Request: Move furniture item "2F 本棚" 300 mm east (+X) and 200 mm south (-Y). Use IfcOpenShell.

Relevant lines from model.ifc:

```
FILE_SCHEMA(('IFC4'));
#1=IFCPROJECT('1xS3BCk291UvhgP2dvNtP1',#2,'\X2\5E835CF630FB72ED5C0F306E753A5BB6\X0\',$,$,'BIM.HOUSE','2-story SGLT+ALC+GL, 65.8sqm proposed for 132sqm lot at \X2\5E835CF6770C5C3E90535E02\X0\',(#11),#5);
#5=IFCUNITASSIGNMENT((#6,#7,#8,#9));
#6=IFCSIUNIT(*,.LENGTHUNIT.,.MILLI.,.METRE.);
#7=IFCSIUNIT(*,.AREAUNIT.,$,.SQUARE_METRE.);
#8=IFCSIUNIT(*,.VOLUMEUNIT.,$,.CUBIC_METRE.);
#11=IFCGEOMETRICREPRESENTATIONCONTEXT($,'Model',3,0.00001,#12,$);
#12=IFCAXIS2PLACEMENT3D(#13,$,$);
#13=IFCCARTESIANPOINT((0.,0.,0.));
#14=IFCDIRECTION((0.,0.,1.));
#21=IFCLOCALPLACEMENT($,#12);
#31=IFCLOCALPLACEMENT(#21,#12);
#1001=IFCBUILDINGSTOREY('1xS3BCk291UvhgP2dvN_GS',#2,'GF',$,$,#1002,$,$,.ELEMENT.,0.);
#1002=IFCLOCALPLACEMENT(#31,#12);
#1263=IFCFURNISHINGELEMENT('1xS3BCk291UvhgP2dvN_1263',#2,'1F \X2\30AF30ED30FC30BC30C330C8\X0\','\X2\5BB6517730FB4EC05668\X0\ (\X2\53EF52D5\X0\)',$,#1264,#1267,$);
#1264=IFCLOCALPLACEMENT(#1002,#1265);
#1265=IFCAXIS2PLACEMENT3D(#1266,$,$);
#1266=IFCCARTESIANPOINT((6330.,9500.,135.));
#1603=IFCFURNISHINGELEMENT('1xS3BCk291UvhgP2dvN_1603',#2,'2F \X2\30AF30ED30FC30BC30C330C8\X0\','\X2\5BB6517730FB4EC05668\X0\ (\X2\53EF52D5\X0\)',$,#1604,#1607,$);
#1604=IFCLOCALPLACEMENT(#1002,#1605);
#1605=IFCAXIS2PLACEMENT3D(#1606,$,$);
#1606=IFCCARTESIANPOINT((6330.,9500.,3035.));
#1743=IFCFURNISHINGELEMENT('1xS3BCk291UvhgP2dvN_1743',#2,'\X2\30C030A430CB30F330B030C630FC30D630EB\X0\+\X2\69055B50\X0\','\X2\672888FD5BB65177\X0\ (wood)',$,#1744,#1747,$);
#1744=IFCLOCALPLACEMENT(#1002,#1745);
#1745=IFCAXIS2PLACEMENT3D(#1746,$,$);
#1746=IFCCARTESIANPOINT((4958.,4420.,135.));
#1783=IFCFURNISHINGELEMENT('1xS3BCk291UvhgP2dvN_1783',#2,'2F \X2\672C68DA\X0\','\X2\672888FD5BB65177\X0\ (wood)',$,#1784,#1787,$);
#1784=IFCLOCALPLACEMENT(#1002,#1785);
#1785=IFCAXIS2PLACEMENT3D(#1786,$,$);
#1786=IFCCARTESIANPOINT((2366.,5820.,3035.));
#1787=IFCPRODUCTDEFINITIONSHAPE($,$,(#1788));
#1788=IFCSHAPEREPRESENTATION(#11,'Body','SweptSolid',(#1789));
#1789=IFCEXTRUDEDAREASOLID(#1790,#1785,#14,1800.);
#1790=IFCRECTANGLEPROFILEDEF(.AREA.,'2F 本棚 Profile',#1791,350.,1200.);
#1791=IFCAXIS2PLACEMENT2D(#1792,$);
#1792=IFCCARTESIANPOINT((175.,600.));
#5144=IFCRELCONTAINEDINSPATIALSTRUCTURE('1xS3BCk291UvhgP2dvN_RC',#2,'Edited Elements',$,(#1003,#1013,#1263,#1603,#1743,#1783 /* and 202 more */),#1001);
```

```python
import ifcopenshell
import ifcopenshell.api.geometry
import ifcopenshell.util.placement
import ifcopenshell.util.unit

model = ifcopenshell.open("model.ifc")
unit_scale = ifcopenshell.util.unit.calculate_unit_scale(model)

item = model.by_guid("1xS3BCk291UvhgP2dvN_1783")
matrix = ifcopenshell.util.placement.get_local_placement(item.ObjectPlacement)
matrix[0, 3] += 0.3 / unit_scale
matrix[1, 3] -= 0.2 / unit_scale
ifcopenshell.api.geometry.edit_object_placement(model, product=item, matrix=matrix, is_si=False)

print(ifcopenshell.util.placement.get_local_placement(item.ObjectPlacement).round(3) + 0.0)

model.write("model_rev.ifc")
```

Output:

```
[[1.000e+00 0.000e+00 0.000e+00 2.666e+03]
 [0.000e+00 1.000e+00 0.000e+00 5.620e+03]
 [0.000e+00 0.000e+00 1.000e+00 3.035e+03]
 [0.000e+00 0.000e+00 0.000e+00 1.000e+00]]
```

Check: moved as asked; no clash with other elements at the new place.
